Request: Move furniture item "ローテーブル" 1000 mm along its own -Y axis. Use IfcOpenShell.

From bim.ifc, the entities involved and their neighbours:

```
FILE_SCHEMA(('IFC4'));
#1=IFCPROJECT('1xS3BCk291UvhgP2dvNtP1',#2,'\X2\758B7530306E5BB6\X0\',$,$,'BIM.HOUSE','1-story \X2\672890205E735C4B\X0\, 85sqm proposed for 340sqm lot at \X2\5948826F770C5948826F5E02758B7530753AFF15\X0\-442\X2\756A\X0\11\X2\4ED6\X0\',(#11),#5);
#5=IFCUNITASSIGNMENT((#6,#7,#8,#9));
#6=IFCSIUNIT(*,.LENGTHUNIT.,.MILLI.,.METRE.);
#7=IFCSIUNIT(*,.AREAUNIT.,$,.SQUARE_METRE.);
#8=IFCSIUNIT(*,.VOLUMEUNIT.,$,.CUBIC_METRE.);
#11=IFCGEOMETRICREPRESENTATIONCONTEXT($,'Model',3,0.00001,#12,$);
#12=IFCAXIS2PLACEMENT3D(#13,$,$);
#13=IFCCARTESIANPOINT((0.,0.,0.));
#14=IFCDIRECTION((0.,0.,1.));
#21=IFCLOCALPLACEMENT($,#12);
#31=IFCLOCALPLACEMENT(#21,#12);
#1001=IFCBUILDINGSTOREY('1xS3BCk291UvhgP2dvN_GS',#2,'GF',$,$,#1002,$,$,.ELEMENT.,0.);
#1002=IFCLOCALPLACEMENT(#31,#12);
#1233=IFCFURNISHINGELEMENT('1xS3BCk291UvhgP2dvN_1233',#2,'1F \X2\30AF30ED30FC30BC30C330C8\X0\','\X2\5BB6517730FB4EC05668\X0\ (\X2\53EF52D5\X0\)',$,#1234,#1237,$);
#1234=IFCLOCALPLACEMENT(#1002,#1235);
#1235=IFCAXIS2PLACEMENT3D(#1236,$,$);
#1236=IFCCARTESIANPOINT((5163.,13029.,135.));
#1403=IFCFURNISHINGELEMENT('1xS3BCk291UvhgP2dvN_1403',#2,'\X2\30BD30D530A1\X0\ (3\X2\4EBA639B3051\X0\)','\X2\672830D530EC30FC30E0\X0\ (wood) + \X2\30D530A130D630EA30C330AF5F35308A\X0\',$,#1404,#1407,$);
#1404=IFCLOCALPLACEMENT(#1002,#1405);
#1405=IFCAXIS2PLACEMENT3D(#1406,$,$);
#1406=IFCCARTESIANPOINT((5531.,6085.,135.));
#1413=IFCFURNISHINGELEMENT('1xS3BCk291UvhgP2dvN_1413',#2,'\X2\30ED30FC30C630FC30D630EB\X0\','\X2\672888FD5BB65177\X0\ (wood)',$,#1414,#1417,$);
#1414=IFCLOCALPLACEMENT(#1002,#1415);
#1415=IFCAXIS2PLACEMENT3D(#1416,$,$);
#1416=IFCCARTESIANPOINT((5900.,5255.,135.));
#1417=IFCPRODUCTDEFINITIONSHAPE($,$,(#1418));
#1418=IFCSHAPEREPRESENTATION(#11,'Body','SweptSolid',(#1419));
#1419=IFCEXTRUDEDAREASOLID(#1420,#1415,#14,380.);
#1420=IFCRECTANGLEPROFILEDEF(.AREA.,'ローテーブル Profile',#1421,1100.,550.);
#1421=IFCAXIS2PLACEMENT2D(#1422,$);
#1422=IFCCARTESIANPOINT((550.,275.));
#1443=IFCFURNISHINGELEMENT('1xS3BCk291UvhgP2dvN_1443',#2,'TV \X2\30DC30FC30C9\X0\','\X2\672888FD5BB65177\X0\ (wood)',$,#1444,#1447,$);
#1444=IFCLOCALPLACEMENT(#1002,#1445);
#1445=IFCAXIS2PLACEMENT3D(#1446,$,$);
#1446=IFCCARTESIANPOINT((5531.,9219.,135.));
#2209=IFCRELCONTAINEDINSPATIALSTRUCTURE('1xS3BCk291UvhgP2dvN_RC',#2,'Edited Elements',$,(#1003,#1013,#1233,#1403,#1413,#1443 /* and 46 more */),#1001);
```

```python
import ifcopenshell
import ifcopenshell.api.geometry
import ifcopenshell.util.placement

model = ifcopenshell.open("bim.ifc")

item = model.by_id(1413)
matrix = ifcopenshell.util.placement.get_local_placement(item.ObjectPlacement)
matrix[:3, 3] -= matrix[:3, 1] * 1000.0
ifcopenshell.api.geometry.edit_object_placement(model, product=item, matrix=matrix, is_si=False)

print(ifcopenshell.util.placement.get_local_placement(item.ObjectPlacement).round(3) + 0.0)

model.write("bim_updated.ifc")
```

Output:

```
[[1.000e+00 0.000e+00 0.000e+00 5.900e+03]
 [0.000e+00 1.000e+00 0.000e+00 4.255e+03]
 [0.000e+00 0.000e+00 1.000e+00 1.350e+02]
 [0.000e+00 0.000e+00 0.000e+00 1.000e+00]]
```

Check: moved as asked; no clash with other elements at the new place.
